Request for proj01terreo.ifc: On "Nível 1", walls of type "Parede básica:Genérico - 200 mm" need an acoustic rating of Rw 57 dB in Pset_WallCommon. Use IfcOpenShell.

First a look at what the model holds.

```python
import ifcopenshell
import ifcopenshell.util.element

model = ifcopenshell.open("proj01terreo.ifc")
print(model.schema)
storey = next(s for s in model.by_type("IfcBuildingStorey") if s.Name == "Nível 1")
walls = [e for e in ifcopenshell.util.element.get_decomposition(storey) if e.is_a("IfcWall")]
seen = {}
for e in walls:
    element_type = ifcopenshell.util.element.get_type(e)
    key = (element_type.Name if element_type != e and element_type else None, ifcopenshell.util.element.get_pset(e, "Pset_WallCommon", "AcousticRating"))
    seen[key] = seen.get(key, 0) + 1
for (name, value), count in sorted(seen.items(), key=str):
    print(count, "x", name, "|", value)
```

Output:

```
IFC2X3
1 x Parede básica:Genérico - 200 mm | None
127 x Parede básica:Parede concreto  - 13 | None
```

```python
import ifcopenshell
import ifcopenshell.api.pset
import ifcopenshell.util.element

model = ifcopenshell.open("proj01terreo.ifc")

storey = next(s for s in model.by_type("IfcBuildingStorey") if s.Name == "Nível 1")
walls = [e for e in ifcopenshell.util.element.get_decomposition(storey) if e.is_a("IfcWall")]

count = 0
for e in walls:
    element_type = ifcopenshell.util.element.get_type(e)
    if element_type in (None, e) or element_type.Name != "Parede básica:Genérico - 200 mm":
        continue
    # add_pset returns the element's existing set when there is one.
    pset = ifcopenshell.api.pset.add_pset(model, product=e, name="Pset_WallCommon")
    ifcopenshell.api.pset.edit_pset(model, pset=pset, properties={"AcousticRating": "Rw 57 dB"})
    count += 1

print(count, "walls updated")

model.write("proj01terreo_rev.ifc")
```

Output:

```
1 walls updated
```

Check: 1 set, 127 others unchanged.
